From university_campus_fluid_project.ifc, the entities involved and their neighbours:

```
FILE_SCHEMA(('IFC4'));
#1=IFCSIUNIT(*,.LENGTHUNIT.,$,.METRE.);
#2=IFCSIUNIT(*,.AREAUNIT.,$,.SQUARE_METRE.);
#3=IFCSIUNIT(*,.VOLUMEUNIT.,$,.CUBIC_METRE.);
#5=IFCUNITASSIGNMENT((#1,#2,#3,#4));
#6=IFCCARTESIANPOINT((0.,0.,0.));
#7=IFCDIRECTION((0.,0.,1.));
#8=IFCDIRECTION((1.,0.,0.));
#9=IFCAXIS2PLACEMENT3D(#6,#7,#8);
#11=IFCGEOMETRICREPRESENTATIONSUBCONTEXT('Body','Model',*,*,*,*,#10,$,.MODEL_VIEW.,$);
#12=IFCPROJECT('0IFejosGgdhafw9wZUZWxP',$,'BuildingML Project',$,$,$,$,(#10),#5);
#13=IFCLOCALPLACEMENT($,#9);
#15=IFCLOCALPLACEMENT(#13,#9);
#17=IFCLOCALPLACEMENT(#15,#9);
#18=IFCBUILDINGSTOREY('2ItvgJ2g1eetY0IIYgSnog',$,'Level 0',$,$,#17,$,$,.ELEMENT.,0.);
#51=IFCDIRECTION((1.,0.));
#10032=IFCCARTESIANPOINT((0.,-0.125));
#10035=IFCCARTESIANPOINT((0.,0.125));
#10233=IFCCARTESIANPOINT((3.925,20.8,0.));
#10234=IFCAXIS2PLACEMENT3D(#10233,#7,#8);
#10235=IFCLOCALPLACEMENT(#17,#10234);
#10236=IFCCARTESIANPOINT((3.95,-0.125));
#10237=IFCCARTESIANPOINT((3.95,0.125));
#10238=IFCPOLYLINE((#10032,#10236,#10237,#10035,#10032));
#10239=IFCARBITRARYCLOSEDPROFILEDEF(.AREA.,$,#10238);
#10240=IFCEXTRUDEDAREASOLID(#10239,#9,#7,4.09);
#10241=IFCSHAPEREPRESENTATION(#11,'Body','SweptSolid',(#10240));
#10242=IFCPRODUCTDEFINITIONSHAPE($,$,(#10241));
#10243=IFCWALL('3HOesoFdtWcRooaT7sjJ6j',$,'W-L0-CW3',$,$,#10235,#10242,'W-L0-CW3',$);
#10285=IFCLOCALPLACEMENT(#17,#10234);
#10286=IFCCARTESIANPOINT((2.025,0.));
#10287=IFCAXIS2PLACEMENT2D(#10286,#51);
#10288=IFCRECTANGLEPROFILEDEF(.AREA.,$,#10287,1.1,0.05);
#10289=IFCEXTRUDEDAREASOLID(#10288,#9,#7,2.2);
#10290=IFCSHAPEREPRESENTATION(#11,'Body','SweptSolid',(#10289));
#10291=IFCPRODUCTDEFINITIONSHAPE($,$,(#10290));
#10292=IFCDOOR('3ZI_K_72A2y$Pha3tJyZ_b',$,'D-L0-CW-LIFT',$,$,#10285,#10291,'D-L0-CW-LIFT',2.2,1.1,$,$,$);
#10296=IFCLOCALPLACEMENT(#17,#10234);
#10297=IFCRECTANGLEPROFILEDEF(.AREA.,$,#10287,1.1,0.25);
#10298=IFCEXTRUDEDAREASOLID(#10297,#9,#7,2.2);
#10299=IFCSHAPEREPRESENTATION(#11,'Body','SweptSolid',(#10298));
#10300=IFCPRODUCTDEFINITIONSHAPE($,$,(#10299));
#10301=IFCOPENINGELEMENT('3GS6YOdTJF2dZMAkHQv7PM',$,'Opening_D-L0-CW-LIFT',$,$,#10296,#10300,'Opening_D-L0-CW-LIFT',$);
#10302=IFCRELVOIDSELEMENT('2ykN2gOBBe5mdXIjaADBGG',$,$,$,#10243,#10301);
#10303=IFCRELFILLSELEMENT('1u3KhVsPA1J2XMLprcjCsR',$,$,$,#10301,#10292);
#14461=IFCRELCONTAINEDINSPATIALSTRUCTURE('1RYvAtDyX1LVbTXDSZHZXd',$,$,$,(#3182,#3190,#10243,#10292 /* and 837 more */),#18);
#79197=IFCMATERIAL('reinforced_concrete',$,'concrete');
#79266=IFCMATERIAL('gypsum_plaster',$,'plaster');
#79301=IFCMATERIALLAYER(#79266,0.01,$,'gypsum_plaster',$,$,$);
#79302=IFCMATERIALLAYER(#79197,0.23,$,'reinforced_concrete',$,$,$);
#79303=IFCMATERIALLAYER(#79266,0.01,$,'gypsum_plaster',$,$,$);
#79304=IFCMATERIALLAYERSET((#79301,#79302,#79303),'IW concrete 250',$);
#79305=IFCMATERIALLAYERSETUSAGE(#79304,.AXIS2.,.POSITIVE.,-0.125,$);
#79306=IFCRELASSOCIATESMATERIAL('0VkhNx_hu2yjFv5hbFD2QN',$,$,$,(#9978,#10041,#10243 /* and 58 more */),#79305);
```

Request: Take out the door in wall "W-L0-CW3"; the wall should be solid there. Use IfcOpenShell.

```python
import ifcopenshell
import ifcopenshell.api.feature
import ifcopenshell.api.root
import ifcopenshell.geom
import ifcopenshell.util.shape

model = ifcopenshell.open("university_campus_fluid_project.ifc")
settings = ifcopenshell.geom.settings()


def volume(element):
    """Net volume in cubic metres, openings subtracted."""
    shape = ifcopenshell.geom.create_shape(settings, element)
    return ifcopenshell.util.shape.get_volume(shape.geometry)


door = model.by_id(10292)
opening = door.FillsVoids[0].RelatingOpeningElement
wall = opening.VoidsElements[0].RelatingBuildingElement
before = volume(wall)

ifcopenshell.api.root.remove_product(model, product=door)
ifcopenshell.api.feature.remove_feature(model, feature=opening)

after = volume(wall)

print(f"wall volume {before:.3f} -> {after:.3f} m3")

model.write("university_campus_fluid_project-out.ifc")
```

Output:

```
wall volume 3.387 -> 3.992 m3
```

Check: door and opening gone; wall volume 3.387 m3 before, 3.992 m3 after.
